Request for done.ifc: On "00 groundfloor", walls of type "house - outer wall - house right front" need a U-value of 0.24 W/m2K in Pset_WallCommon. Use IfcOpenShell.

First a look at what the model holds.

```python
import ifcopenshell
import ifcopenshell.util.element

model = ifcopenshell.open("done.ifc")
print(model.schema)
storey = next(s for s in model.by_type("IfcBuildingStorey") if s.Name == "00 groundfloor")
walls = [e for e in ifcopenshell.util.element.get_decomposition(storey) if e.is_a("IfcWall")]
seen = {}
for e in walls:
    element_type = ifcopenshell.util.element.get_type(e)
    key = (element_type.Name if element_type != e and element_type else None, ifcopenshell.util.element.get_pset(e, "Pset_WallCommon", "ThermalTransmittance"))
    seen[key] = seen.get(key, 0) + 1
for (name, value), count in sorted(seen.items(), key=str):
    print(count, "x", name, "|", value)
```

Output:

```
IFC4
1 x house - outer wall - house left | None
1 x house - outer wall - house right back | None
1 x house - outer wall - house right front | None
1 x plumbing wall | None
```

```python
import ifcopenshell
import ifcopenshell.api.pset
import ifcopenshell.util.element

model = ifcopenshell.open("done.ifc")

storey = next(s for s in model.by_type("IfcBuildingStorey") if s.Name == "00 groundfloor")
walls = [e for e in ifcopenshell.util.element.get_decomposition(storey) if e.is_a("IfcWall")]

count = 0
for e in walls:
    element_type = ifcopenshell.util.element.get_type(e)
    if element_type in (None, e) or element_type.Name != "house - outer wall - house right front":
        continue
    # add_pset returns the element's existing set when there is one.
    pset = ifcopenshell.api.pset.add_pset(model, product=e, name="Pset_WallCommon")
    ifcopenshell.api.pset.edit_pset(model, pset=pset, properties={"ThermalTransmittance": 0.24})
    count += 1

print(count, "walls updated")

model.write("done_v2.ifc")
```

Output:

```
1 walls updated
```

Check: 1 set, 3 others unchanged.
